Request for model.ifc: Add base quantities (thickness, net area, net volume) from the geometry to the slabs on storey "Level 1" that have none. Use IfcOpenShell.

First a look at what the model holds.

```python
import ifcopenshell
import ifcopenshell.util.element
import ifcopenshell.util.unit

model = ifcopenshell.open("model.ifc")
print(model.schema)
for unit_type in ("LENGTHUNIT", "AREAUNIT", "VOLUMEUNIT"):
    print(unit_type, ifcopenshell.util.unit.calculate_unit_scale(model, unit_type))
storey = next(s for s in model.by_type("IfcBuildingStorey") if s.Name == "Level 1")
slabs = [e for e in ifcopenshell.util.element.get_decomposition(storey) if e.is_a("IfcSlab")]
for e in sorted(slabs, key=lambda e: e.id()):
    print(e.id(), e.is_a(), e.Name, list(ifcopenshell.util.element.get_psets(e, qtos_only=True)), sep=" | ")
```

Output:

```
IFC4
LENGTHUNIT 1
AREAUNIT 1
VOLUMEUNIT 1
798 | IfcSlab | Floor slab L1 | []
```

```python
import ifcopenshell
import ifcopenshell.api.pset
import ifcopenshell.geom
import ifcopenshell.util.element
import ifcopenshell.util.shape
import ifcopenshell.util.unit

model = ifcopenshell.open("model.ifc")
unit_scale = ifcopenshell.util.unit.calculate_unit_scale(model)
area_scale = ifcopenshell.util.unit.calculate_unit_scale(model, "AREAUNIT")
volume_scale = ifcopenshell.util.unit.calculate_unit_scale(model, "VOLUMEUNIT")
settings = ifcopenshell.geom.settings()

storey = next(s for s in model.by_type("IfcBuildingStorey") if s.Name == "Level 1")
slabs = [e for e in ifcopenshell.util.element.get_decomposition(storey) if e.is_a("IfcSlab")]

for e in sorted(slabs, key=lambda e: e.id()):
    if ifcopenshell.util.element.get_psets(e, qtos_only=True, should_inherit=False):
        continue
    # Geometry comes back in metres, in the element's own axes.
    shape = ifcopenshell.geom.create_shape(settings, e)
    values = {
        "Width": ifcopenshell.util.shape.get_z(shape.geometry) / unit_scale,
        "NetArea": ifcopenshell.util.shape.get_footprint_area(shape.geometry) / area_scale,
        "NetVolume": ifcopenshell.util.shape.get_volume(shape.geometry) / volume_scale,
    }
    qto = ifcopenshell.api.pset.add_qto(model, product=e, name="Qto_SlabBaseQuantities")
    ifcopenshell.api.pset.edit_qto(model, qto=qto, properties=values)
    print(e.id(), {k: round(v, 3) for k, v in values.items()})

model.write("model_edited.ifc")
```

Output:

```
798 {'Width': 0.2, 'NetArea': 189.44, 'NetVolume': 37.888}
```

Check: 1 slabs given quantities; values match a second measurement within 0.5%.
